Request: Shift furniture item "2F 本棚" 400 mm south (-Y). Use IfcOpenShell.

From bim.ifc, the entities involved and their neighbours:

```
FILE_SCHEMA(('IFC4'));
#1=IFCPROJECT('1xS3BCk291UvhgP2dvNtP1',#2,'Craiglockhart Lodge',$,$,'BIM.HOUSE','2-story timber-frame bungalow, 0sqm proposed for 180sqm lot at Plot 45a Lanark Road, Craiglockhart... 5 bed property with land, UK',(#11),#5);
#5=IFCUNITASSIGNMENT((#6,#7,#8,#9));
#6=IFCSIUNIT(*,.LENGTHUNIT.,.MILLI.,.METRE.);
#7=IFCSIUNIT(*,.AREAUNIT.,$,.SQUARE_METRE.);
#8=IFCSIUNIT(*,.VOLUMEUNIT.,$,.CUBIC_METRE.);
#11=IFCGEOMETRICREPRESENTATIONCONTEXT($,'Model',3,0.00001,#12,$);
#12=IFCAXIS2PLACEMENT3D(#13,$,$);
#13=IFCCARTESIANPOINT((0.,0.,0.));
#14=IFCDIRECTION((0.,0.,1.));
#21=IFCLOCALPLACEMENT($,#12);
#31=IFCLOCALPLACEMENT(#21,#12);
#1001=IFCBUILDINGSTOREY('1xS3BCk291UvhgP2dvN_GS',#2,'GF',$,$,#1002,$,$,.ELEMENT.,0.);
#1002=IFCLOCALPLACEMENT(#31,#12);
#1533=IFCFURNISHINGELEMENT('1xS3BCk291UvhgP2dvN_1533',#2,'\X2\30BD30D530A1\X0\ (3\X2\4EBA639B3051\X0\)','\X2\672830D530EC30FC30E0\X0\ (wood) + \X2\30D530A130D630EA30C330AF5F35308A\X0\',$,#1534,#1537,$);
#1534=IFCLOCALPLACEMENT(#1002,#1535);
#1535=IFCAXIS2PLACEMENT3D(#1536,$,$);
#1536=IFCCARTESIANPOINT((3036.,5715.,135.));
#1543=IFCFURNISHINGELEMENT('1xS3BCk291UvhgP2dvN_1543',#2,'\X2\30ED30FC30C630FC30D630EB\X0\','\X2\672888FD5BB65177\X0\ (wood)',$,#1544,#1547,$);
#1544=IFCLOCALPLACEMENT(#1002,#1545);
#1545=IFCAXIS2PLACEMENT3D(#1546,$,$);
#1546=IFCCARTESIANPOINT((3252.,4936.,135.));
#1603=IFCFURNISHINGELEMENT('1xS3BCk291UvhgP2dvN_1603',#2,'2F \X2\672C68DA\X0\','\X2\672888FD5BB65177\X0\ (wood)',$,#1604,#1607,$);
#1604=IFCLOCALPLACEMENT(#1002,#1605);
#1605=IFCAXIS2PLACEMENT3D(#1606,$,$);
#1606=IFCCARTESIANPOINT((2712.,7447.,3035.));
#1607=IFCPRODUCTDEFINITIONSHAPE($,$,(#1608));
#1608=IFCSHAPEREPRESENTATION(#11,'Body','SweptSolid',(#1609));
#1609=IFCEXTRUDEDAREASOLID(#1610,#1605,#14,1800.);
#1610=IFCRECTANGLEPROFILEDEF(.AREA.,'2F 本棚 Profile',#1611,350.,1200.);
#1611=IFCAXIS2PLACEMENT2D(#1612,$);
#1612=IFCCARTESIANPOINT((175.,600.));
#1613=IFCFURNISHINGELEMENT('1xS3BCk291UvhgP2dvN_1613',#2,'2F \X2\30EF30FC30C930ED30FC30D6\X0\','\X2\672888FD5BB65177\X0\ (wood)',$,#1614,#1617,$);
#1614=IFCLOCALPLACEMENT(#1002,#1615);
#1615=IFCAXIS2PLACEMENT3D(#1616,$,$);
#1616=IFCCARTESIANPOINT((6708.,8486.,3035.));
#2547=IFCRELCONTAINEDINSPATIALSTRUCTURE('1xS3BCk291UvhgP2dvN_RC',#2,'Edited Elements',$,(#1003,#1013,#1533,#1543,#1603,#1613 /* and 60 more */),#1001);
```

```python
import ifcopenshell
import ifcopenshell.api.geometry
import ifcopenshell.util.placement

model = ifcopenshell.open("bim.ifc")

item = model.by_guid("1xS3BCk291UvhgP2dvN_1603")
matrix = ifcopenshell.util.placement.get_local_placement(item.ObjectPlacement)
matrix[1, 3] -= 400.0
ifcopenshell.api.geometry.edit_object_placement(model, product=item, matrix=matrix, is_si=False)

print(ifcopenshell.util.placement.get_local_placement(item.ObjectPlacement).round(3) + 0.0)

model.write("bim_edited.ifc")
```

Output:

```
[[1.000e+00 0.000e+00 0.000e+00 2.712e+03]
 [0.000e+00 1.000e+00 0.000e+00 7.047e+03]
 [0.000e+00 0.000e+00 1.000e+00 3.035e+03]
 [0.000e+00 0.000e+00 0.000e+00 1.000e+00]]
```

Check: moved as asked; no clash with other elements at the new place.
